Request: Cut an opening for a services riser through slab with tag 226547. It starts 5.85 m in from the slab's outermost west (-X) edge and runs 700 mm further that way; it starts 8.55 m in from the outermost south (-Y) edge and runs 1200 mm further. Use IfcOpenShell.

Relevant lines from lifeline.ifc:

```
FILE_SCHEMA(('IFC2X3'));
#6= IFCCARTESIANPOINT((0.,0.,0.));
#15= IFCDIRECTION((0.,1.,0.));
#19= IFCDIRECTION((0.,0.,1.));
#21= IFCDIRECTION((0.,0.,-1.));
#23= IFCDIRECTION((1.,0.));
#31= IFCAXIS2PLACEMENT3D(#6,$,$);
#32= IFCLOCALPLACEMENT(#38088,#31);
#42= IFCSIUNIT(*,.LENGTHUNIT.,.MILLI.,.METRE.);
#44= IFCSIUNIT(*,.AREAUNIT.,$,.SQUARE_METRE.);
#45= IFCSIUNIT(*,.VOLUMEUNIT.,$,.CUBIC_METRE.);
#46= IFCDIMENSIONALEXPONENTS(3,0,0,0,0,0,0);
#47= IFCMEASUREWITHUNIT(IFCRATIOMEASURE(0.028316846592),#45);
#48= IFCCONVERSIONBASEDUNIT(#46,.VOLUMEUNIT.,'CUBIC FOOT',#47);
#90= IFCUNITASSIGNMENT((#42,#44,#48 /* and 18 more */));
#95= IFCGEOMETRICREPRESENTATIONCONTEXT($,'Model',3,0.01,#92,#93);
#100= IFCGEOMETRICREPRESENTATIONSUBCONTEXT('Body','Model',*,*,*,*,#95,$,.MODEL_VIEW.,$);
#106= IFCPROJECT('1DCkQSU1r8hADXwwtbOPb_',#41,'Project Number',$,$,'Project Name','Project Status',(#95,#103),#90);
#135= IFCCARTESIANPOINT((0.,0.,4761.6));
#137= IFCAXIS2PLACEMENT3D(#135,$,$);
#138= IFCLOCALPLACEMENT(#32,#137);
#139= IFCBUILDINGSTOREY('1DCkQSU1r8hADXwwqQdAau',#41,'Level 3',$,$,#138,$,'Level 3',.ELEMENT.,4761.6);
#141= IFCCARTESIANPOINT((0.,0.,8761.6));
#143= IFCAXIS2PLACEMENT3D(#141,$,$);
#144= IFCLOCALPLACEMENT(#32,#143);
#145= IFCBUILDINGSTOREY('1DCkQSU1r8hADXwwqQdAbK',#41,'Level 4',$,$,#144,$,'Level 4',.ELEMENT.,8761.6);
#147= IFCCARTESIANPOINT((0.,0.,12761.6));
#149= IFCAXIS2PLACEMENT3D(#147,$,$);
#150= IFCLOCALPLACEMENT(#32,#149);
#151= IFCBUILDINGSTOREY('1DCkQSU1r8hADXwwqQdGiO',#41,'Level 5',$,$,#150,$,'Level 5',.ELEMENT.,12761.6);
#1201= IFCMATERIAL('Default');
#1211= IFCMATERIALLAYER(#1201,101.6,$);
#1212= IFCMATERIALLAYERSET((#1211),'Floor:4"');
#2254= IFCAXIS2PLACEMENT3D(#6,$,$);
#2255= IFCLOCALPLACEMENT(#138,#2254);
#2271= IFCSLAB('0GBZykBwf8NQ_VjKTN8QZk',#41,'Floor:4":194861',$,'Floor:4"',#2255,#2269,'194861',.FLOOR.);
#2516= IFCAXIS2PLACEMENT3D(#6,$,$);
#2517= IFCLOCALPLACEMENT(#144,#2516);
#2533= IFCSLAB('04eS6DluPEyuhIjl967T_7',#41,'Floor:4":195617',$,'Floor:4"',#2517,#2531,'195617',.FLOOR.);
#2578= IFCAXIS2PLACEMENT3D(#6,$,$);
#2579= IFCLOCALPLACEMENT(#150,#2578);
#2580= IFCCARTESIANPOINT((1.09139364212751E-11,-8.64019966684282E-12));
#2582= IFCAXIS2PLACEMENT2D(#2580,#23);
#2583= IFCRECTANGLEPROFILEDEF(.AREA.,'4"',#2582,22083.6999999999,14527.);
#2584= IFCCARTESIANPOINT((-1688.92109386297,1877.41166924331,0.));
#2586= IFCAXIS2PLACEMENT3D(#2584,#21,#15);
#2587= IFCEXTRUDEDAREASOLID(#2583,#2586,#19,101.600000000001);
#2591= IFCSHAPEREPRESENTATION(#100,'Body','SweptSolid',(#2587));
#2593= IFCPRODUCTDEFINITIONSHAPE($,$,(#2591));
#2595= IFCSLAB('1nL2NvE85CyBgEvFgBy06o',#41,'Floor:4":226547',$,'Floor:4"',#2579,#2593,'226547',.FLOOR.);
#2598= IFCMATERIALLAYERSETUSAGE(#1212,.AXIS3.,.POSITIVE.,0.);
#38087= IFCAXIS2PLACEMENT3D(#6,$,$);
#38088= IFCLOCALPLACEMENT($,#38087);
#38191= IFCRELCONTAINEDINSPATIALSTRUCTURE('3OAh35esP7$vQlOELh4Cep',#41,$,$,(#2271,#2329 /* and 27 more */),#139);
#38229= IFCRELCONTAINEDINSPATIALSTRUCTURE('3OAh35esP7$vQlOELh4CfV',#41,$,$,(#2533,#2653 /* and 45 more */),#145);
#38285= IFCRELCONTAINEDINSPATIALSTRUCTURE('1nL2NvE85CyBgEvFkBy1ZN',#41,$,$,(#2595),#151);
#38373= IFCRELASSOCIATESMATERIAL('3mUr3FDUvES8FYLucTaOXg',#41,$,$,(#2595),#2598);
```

```python
import numpy as np
import ifcopenshell
import ifcopenshell.api.feature
import ifcopenshell.api.geometry
import ifcopenshell.api.root
import ifcopenshell.geom
import ifcopenshell.util.placement
import ifcopenshell.util.representation
import ifcopenshell.util.shape
import ifcopenshell.util.unit

model = ifcopenshell.open("lifeline.ifc")
unit_scale = ifcopenshell.util.unit.calculate_unit_scale(model)
settings = ifcopenshell.geom.settings()


def volume(element):
    """Net volume in cubic metres, openings subtracted."""
    shape = ifcopenshell.geom.create_shape(settings, element)
    return ifcopenshell.util.shape.get_volume(shape.geometry)


slab = model.by_guid("1nL2NvE85CyBgEvFgBy06o")
before = volume(slab)

# Extent in the slab's own axes, in metres. The edges named are its -X and -Y sides.
slab_shape = ifcopenshell.geom.create_shape(settings, slab)
vertices = ifcopenshell.util.shape.get_vertices(slab_shape.geometry)
x_min, y_min, bottom = vertices.min(axis=0)
top = vertices[:, 2].max()

opening = ifcopenshell.api.root.create_entity(model, ifc_class="IfcOpeningElement", name="Services riser opening")
context = ifcopenshell.util.representation.get_context(model, "Model", "Body", "MODEL_VIEW")
width, depth = 0.7, 1.2
outline = [(0.0, 0.0), (width, 0.0), (width, depth), (0.0, depth), (0.0, 0.0)]
# Overshoot both faces by 50 mm so the cut is clean.
shape = ifcopenshell.api.geometry.add_slab_representation(
    model, context=context, depth=top - bottom + 0.1, polyline=outline
)
ifcopenshell.api.geometry.assign_representation(model, product=opening, representation=shape)

matrix = ifcopenshell.util.placement.get_local_placement(slab.ObjectPlacement)
matrix[:, 3] = matrix @ np.append(np.array([x_min + 5.85, y_min + 8.55, bottom - 0.05]) / unit_scale, 1.0)
ifcopenshell.api.geometry.edit_object_placement(model, product=opening, matrix=matrix, is_si=False)
ifcopenshell.api.feature.add_feature(model, feature=opening, element=slab)

after = volume(slab)

print(f"slab volume {before:.3f} -> {after:.3f} m3")

model.write("lifeline_updated.ifc")
```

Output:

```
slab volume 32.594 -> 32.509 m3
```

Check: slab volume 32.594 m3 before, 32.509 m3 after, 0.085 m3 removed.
